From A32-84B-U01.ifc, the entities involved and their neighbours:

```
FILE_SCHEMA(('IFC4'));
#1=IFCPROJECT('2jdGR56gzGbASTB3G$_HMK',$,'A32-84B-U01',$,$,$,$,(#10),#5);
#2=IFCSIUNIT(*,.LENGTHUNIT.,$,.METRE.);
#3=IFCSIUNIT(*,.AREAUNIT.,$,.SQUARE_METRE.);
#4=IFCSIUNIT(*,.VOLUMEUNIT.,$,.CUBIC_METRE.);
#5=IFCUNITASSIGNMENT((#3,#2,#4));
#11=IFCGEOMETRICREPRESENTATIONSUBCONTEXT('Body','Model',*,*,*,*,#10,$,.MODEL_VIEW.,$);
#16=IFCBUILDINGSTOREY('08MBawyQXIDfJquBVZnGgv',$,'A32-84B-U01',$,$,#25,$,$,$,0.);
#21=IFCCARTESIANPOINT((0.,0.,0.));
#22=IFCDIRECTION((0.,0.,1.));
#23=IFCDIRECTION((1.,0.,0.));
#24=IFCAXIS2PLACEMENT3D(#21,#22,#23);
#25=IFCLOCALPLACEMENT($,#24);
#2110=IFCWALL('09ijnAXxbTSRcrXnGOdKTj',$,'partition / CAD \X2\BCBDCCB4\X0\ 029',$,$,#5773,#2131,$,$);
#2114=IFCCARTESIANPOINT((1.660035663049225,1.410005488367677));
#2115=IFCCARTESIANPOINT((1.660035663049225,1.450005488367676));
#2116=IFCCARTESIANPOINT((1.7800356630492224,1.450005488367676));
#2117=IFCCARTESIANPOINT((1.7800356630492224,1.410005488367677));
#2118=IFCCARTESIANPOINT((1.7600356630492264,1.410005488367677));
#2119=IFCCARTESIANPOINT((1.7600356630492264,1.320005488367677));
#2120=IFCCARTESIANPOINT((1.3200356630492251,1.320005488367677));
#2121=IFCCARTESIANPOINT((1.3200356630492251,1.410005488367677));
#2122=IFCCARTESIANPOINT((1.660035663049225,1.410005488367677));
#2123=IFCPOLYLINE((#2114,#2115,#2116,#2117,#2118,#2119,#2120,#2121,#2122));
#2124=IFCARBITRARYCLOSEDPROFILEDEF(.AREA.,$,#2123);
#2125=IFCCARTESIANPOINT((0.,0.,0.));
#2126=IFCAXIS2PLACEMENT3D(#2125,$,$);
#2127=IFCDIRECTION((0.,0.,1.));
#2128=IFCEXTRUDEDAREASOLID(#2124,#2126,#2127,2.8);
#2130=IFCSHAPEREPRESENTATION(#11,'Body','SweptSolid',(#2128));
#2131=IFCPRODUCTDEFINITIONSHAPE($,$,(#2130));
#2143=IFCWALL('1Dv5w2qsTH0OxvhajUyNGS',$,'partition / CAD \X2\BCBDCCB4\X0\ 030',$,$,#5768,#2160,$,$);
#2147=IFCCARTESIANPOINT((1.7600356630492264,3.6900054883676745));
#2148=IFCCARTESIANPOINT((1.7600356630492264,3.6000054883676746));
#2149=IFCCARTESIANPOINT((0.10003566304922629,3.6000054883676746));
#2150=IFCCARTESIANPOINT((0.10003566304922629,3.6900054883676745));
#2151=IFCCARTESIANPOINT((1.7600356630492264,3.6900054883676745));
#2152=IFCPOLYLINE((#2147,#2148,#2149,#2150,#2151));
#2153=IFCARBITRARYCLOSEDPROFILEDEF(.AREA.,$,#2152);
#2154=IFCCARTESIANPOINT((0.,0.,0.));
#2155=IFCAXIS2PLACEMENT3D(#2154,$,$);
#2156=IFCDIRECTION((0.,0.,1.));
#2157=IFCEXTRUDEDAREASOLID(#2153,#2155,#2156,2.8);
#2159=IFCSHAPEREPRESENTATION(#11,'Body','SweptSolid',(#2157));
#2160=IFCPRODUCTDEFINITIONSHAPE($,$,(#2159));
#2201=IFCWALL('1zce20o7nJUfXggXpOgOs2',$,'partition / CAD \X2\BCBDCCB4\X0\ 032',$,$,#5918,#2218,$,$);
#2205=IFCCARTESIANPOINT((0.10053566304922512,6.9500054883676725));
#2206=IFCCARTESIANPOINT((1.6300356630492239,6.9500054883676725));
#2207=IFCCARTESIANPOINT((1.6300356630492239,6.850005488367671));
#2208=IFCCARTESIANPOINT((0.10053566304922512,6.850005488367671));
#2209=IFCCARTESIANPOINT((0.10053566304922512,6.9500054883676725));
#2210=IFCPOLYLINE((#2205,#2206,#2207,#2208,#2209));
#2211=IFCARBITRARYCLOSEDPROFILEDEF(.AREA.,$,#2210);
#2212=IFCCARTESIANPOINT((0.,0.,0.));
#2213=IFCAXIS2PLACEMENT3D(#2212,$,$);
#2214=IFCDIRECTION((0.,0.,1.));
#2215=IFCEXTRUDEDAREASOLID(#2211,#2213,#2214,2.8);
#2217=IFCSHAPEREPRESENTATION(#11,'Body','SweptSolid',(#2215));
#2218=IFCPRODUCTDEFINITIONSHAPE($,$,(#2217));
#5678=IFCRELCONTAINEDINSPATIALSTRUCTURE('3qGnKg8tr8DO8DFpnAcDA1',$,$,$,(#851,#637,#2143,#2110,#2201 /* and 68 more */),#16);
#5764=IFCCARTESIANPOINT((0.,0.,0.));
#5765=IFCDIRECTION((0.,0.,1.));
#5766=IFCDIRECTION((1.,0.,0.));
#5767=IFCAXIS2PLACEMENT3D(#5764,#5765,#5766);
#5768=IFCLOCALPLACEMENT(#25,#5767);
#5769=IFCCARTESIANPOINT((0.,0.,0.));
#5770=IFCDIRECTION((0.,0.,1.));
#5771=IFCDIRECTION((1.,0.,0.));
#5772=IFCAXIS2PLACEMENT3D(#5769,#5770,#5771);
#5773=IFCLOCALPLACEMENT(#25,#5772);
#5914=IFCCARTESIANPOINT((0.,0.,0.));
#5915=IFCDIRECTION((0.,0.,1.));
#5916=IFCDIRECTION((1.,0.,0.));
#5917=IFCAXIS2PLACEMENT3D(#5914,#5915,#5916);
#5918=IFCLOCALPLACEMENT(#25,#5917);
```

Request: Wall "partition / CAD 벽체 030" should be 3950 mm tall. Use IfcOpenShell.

```python
import ifcopenshell
import ifcopenshell.geom
import ifcopenshell.util.representation
import ifcopenshell.util.shape

model = ifcopenshell.open("A32-84B-U01.ifc")
settings = ifcopenshell.geom.settings()


def volume(element):
    """Net volume in cubic metres, openings subtracted."""
    shape = ifcopenshell.geom.create_shape(settings, element)
    return ifcopenshell.util.shape.get_volume(shape.geometry)


wall = model.by_guid("1Dv5w2qsTH0OxvhajUyNGS")
before = volume(wall)

body = ifcopenshell.util.representation.get_representation(wall, "Model", "Body")
solid = body.Items[0]
old_height = solid.Depth
solid.Depth = 3.95
after = volume(wall)

print(f"height {old_height:g} -> {solid.Depth:g}, volume {before:.3f} -> {after:.3f} m3")

model.write("A32-84B-U01_rev.ifc")
```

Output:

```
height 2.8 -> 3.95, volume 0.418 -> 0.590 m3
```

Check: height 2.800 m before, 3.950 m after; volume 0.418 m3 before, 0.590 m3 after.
